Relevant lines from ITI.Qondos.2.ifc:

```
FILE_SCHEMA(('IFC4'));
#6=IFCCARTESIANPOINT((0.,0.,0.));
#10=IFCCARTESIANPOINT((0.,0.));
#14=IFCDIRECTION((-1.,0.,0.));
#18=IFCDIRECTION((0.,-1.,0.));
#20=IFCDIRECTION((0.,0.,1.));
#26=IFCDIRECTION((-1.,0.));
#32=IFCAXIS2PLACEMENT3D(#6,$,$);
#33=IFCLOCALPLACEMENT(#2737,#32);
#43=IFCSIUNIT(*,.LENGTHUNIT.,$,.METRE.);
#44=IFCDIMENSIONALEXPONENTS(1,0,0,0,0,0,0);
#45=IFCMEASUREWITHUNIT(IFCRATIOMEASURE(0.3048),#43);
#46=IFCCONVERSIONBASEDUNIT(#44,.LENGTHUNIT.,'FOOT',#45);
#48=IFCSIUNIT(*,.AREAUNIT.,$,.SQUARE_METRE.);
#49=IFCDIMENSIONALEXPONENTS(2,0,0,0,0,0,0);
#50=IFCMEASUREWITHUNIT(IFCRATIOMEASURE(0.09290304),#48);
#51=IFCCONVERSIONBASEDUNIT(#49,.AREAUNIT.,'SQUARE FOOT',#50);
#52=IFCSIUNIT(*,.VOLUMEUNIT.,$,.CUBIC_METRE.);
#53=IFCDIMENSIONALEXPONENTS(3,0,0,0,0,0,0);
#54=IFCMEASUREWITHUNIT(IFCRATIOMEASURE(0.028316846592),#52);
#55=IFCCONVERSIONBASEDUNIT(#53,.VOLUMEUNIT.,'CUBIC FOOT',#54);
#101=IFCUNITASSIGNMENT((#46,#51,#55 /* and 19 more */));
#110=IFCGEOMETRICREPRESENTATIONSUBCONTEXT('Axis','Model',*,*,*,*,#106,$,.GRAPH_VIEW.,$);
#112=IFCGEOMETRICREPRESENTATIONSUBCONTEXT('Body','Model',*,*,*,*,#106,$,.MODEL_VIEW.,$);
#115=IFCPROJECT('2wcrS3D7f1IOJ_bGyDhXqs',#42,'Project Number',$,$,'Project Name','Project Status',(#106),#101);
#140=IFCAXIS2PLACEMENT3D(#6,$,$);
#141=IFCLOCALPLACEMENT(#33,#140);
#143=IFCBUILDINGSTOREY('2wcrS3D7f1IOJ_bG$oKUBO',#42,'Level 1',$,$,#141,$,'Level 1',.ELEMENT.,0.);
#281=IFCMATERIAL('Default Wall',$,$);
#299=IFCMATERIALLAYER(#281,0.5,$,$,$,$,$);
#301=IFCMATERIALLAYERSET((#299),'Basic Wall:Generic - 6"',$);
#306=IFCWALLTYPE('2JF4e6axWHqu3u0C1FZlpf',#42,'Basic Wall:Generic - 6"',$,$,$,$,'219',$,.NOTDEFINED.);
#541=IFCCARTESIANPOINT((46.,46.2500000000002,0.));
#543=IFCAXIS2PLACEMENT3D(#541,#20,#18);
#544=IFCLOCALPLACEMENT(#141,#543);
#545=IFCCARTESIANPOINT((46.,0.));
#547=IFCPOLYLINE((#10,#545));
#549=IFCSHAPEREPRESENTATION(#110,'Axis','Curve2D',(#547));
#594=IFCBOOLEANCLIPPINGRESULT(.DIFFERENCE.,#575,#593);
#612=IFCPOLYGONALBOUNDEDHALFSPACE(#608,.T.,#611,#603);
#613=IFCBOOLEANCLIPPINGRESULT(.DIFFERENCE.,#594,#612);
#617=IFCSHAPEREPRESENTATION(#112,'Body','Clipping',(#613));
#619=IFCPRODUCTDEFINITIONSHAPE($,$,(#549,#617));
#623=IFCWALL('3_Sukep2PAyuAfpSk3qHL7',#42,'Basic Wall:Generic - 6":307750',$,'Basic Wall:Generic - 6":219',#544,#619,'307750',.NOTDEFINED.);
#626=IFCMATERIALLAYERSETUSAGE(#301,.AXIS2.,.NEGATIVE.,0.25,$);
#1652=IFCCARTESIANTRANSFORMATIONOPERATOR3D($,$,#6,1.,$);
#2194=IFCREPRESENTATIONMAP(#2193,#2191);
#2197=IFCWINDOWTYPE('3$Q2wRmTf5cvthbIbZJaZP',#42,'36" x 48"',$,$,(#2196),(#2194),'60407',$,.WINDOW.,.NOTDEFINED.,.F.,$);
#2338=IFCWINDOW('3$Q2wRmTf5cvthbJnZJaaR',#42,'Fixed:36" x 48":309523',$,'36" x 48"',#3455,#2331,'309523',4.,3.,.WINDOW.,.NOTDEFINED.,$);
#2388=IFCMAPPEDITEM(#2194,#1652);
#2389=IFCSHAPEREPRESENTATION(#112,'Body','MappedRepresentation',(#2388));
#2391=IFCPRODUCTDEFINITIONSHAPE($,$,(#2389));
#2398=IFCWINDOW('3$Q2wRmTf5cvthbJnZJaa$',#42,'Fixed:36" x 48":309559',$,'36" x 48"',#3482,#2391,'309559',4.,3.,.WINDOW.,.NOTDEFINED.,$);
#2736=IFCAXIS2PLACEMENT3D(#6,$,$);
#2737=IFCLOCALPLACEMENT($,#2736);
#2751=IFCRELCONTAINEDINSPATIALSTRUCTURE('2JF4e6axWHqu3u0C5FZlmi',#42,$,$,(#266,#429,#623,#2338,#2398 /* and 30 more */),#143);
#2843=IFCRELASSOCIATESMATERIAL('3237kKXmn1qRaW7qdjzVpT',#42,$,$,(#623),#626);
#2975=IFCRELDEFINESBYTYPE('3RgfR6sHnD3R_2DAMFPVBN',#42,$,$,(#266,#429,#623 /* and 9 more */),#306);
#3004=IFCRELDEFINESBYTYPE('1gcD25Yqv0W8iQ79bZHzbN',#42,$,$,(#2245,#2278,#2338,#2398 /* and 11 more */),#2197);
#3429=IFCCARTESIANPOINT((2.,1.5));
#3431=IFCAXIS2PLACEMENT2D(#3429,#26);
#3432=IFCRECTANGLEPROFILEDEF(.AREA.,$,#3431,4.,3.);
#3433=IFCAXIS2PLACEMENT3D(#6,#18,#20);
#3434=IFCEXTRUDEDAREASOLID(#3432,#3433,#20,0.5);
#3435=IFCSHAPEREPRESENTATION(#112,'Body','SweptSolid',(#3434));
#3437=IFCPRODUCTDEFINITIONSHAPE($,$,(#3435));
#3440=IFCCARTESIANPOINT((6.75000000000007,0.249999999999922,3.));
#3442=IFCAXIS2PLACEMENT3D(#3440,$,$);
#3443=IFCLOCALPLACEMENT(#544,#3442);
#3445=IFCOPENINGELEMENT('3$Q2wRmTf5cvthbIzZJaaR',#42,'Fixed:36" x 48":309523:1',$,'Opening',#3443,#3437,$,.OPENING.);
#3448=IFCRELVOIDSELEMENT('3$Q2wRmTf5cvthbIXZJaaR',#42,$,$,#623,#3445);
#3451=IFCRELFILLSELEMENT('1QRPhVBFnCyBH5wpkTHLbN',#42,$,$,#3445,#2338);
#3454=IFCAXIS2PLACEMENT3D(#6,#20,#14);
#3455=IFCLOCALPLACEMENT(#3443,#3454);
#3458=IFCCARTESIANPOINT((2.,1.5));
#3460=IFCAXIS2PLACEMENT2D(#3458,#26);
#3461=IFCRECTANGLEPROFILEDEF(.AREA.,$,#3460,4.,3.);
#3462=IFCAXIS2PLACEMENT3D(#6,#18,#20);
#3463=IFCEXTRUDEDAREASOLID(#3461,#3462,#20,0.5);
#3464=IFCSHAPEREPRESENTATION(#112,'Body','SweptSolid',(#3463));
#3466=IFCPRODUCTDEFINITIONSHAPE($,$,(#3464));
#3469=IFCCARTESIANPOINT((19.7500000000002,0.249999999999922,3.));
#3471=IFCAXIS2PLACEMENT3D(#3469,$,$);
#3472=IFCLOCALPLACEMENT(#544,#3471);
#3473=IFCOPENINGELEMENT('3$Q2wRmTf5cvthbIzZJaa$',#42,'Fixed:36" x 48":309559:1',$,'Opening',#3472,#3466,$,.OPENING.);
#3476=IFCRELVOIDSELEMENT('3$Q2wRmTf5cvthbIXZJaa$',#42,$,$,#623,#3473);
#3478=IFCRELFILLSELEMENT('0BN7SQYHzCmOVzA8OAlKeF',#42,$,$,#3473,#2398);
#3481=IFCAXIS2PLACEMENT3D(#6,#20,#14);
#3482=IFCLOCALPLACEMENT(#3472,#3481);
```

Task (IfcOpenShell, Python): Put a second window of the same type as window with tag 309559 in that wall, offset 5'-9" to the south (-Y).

```python
import ifcopenshell
import ifcopenshell.api.feature
import ifcopenshell.api.geometry
import ifcopenshell.api.root
import ifcopenshell.geom
import ifcopenshell.util.element
import ifcopenshell.util.placement
import ifcopenshell.util.shape
import ifcopenshell.util.unit

model = ifcopenshell.open("ITI.Qondos.2.ifc")
unit_scale = ifcopenshell.util.unit.calculate_unit_scale(model)
settings = ifcopenshell.geom.settings()


def volume(element):
    """Net volume in cubic metres, openings subtracted."""
    shape = ifcopenshell.geom.create_shape(settings, element)
    return ifcopenshell.util.shape.get_volume(shape.geometry)


def reuse_history(source, copy):
    """copy_class also copies each property set's owner history, people and application; keep the originals."""
    for rel in copy.IsDefinedBy:
        if rel.is_a("IfcRelDefinesByProperties") and (history := rel.RelatingPropertyDefinition.OwnerHistory):
            rel.RelatingPropertyDefinition.OwnerHistory = source.OwnerHistory
            ifcopenshell.util.element.remove_deep2(model, history)


window = model.by_guid("3$Q2wRmTf5cvthbJnZJaa$")
opening = window.FillsVoids[0].RelatingOpeningElement
wall = opening.VoidsElements[0].RelatingBuildingElement
before = volume(wall)
shift = ifcopenshell.util.placement.get_local_placement(wall.ObjectPlacement)[:3, 0] * 69 * 0.0254 / unit_scale

# copy_class copies the void relationship, type, container and properties, but no geometry.
new_opening = ifcopenshell.api.root.copy_class(model, product=opening)
new_opening.Representation = ifcopenshell.util.element.copy_deep(
    model, opening.Representation, exclude=["IfcGeometricRepresentationContext", "IfcRepresentationMap"]
)
new_opening.Name = 'Fixed:36" x 48"'
new_window = ifcopenshell.api.root.copy_class(model, product=window)
new_window.Representation = ifcopenshell.util.element.copy_deep(
    model, window.Representation, exclude=["IfcGeometricRepresentationContext", "IfcRepresentationMap"]
)
new_window.Name = 'Fixed:36" x 48"'
new_window.Tag = None
reuse_history(window, new_window)
ifcopenshell.api.feature.add_filling(model, opening=new_opening, element=new_window)

for old, new in ((opening, new_opening), (window, new_window)):
    matrix = ifcopenshell.util.placement.get_local_placement(old.ObjectPlacement)
    matrix[:3, 3] += shift
    ifcopenshell.api.geometry.edit_object_placement(model, product=new, matrix=matrix, is_si=False)

after = volume(wall)

print(f"wall volume {before:.3f} -> {after:.3f} m3")

model.write("ITI.Qondos.2_edited.ifc")
```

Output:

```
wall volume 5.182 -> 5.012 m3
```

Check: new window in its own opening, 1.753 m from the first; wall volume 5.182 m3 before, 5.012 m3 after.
